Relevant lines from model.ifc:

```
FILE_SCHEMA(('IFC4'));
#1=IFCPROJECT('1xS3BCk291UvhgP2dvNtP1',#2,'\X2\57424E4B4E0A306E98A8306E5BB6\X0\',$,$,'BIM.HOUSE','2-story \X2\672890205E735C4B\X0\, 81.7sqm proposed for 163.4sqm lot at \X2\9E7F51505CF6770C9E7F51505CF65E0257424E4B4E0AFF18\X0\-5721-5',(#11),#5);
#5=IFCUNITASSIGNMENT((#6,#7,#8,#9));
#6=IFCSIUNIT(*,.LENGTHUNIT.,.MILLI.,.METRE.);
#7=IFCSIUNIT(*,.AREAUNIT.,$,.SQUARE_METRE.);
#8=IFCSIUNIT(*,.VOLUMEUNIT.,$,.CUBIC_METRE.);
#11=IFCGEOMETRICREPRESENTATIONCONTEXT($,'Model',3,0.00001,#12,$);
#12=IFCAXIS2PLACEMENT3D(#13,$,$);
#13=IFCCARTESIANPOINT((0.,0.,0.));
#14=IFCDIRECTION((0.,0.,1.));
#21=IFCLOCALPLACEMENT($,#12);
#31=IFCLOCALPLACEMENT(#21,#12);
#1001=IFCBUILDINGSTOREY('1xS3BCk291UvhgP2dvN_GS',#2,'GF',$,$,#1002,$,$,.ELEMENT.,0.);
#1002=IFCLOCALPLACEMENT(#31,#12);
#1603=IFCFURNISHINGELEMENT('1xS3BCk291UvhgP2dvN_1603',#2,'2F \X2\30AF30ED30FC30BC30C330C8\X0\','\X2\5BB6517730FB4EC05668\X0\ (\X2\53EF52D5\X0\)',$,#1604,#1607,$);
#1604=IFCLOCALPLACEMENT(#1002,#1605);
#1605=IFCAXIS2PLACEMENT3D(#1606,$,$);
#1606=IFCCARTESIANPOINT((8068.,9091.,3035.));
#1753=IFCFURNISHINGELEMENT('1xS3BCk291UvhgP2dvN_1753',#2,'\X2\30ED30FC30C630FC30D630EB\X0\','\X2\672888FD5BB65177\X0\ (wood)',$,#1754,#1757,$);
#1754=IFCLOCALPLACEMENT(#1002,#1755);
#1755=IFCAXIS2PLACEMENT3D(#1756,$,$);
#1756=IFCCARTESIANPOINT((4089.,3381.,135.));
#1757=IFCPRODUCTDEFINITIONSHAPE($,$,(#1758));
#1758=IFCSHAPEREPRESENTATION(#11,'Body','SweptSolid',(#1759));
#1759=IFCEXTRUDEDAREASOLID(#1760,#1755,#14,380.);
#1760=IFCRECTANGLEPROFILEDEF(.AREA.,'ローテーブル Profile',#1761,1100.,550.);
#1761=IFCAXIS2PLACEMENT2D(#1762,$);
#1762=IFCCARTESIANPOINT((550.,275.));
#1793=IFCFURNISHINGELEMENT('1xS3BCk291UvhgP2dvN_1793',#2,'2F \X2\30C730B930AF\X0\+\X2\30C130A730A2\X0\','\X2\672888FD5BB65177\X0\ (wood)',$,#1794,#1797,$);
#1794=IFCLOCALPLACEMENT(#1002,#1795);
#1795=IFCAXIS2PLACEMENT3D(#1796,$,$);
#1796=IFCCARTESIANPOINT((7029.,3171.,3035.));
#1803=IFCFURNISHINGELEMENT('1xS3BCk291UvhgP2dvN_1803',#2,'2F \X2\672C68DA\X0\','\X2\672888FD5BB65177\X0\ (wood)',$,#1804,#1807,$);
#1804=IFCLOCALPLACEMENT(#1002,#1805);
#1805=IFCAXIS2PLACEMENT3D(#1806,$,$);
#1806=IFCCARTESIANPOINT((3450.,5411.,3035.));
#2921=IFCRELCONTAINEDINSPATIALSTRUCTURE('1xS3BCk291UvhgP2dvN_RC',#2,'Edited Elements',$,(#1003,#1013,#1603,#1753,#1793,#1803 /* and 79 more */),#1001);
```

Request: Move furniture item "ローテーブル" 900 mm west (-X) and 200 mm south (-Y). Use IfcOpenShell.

```python
import ifcopenshell
import ifcopenshell.api.geometry
import ifcopenshell.util.placement
import ifcopenshell.util.unit

model = ifcopenshell.open("model.ifc")
unit_scale = ifcopenshell.util.unit.calculate_unit_scale(model)

item = model.by_id(1753)
matrix = ifcopenshell.util.placement.get_local_placement(item.ObjectPlacement)
matrix[0, 3] -= 0.9 / unit_scale
matrix[1, 3] -= 0.2 / unit_scale
ifcopenshell.api.geometry.edit_object_placement(model, product=item, matrix=matrix, is_si=False)

print(ifcopenshell.util.placement.get_local_placement(item.ObjectPlacement).round(3) + 0.0)

model.write("model_rev.ifc")
```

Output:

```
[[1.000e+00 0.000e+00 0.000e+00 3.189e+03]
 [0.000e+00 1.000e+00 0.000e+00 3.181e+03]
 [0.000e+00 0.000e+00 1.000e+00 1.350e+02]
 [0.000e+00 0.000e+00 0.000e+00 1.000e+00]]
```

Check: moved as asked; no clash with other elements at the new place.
